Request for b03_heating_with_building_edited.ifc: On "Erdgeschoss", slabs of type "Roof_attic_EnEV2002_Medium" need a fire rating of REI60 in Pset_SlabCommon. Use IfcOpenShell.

First a look at what the model holds.

```python
import ifcopenshell
import ifcopenshell.util.element

model = ifcopenshell.open("b03_heating_with_building_edited.ifc")
print(model.schema)
storey = next(s for s in model.by_type("IfcBuildingStorey") if s.Name == "Erdgeschoss")
slabs = [e for e in ifcopenshell.util.element.get_decomposition(storey) if e.is_a("IfcSlab")]
seen = {}
for e in slabs:
    element_type = ifcopenshell.util.element.get_type(e)
    key = (element_type.Name if element_type != e and element_type else None, ifcopenshell.util.element.get_pset(e, "Pset_SlabCommon", "FireRating"))
    seen[key] = seen.get(key, 0) + 1
for (name, value), count in sorted(seen.items(), key=str):
    print(count, "x", name, "|", value)
```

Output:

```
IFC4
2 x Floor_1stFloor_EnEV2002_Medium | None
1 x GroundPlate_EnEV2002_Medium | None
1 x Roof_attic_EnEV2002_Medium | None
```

```python
import ifcopenshell
import ifcopenshell.api.pset
import ifcopenshell.util.element

model = ifcopenshell.open("b03_heating_with_building_edited.ifc")

storey = next(s for s in model.by_type("IfcBuildingStorey") if s.Name == "Erdgeschoss")
slabs = [e for e in ifcopenshell.util.element.get_decomposition(storey) if e.is_a("IfcSlab")]

count = 0
for e in slabs:
    element_type = ifcopenshell.util.element.get_type(e)
    if element_type in (None, e) or element_type.Name != "Roof_attic_EnEV2002_Medium":
        continue
    # add_pset returns the element's existing set when there is one.
    pset = ifcopenshell.api.pset.add_pset(model, product=e, name="Pset_SlabCommon")
    ifcopenshell.api.pset.edit_pset(model, pset=pset, properties={"FireRating": "REI60"})
    count += 1

print(count, "slabs updated")

model.write("b03_heating_with_building_edited_updated.ifc")
```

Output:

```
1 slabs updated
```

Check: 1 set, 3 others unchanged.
